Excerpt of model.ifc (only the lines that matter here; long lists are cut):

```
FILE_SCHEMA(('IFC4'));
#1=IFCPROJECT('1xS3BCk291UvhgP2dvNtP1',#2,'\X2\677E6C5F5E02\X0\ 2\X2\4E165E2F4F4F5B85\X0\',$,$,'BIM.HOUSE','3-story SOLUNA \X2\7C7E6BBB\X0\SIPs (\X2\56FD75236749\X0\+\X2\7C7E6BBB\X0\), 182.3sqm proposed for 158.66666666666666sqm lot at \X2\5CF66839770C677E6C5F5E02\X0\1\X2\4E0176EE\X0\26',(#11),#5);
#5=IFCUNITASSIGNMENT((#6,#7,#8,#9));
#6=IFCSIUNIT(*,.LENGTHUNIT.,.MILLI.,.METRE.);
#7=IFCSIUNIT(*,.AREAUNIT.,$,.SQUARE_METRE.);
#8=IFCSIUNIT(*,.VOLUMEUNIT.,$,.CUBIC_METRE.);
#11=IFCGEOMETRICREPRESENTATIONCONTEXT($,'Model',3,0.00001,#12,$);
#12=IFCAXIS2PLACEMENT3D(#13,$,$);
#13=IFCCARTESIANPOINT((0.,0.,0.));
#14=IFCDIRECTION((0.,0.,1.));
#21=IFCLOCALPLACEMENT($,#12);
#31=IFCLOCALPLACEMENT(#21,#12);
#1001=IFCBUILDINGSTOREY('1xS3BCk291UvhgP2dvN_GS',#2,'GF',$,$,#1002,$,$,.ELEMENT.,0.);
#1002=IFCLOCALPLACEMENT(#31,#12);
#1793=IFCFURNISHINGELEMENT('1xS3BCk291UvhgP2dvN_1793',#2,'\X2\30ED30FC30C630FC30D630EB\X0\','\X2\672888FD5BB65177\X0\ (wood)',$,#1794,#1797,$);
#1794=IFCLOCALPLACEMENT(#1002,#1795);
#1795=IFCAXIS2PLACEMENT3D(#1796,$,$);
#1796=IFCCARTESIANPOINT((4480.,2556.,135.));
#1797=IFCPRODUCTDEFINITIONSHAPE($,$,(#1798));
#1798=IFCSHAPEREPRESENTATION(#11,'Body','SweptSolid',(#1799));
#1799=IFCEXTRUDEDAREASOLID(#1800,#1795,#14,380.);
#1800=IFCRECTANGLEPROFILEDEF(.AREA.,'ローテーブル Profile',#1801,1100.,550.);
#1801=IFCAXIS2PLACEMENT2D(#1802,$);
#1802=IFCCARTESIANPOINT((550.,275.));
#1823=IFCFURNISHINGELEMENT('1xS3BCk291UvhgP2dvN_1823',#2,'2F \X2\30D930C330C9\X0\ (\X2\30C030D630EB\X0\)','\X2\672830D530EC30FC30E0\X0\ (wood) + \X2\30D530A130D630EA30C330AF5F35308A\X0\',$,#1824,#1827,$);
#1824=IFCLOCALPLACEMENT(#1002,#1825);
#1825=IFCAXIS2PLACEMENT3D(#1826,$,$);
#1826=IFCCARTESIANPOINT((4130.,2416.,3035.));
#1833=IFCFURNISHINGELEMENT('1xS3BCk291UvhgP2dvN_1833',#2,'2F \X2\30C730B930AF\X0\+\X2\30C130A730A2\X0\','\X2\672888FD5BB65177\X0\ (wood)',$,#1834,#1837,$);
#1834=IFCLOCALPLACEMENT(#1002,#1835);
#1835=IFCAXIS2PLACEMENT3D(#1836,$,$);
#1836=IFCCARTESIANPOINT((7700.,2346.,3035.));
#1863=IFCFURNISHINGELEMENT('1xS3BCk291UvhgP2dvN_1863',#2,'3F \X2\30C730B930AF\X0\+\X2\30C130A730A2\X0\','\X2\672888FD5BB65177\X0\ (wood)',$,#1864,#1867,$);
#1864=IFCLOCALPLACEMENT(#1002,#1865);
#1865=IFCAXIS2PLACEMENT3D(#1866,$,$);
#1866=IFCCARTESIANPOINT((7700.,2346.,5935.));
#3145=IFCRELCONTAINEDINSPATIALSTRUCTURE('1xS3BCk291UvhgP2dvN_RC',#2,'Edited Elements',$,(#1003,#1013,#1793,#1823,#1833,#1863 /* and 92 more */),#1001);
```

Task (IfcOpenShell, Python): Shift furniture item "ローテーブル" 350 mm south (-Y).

```python
import ifcopenshell
import ifcopenshell.api.geometry
import ifcopenshell.util.placement

model = ifcopenshell.open("model.ifc")

item = model.by_guid("1xS3BCk291UvhgP2dvN_1793")
matrix = ifcopenshell.util.placement.get_local_placement(item.ObjectPlacement)
matrix[1, 3] -= 350.0
ifcopenshell.api.geometry.edit_object_placement(model, product=item, matrix=matrix, is_si=False)

print(ifcopenshell.util.placement.get_local_placement(item.ObjectPlacement).round(3) + 0.0)

model.write("model-out.ifc")
```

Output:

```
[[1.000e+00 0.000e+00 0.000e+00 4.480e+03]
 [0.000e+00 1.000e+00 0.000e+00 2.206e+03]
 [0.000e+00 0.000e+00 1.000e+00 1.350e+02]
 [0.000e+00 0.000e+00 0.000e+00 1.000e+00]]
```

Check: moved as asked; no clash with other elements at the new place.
